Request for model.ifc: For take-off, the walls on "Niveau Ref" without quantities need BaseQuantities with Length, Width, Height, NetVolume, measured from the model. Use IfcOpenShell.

First a look at what the model holds.

```python
import ifcopenshell
import ifcopenshell.util.element
import ifcopenshell.util.unit

model = ifcopenshell.open("model.ifc")
print(model.schema)
for unit_type in ("LENGTHUNIT", "AREAUNIT", "VOLUMEUNIT"):
    print(unit_type, ifcopenshell.util.unit.calculate_unit_scale(model, unit_type))
storey = next(s for s in model.by_type("IfcBuildingStorey") if s.Name == "Niveau Ref")
walls = [e for e in ifcopenshell.util.element.get_decomposition(storey) if e.is_a("IfcWall")]
for e in sorted(walls, key=lambda e: e.id()):
    print(e.id(), e.is_a(), e.Name, list(ifcopenshell.util.element.get_psets(e, qtos_only=True)), sep=" | ")
```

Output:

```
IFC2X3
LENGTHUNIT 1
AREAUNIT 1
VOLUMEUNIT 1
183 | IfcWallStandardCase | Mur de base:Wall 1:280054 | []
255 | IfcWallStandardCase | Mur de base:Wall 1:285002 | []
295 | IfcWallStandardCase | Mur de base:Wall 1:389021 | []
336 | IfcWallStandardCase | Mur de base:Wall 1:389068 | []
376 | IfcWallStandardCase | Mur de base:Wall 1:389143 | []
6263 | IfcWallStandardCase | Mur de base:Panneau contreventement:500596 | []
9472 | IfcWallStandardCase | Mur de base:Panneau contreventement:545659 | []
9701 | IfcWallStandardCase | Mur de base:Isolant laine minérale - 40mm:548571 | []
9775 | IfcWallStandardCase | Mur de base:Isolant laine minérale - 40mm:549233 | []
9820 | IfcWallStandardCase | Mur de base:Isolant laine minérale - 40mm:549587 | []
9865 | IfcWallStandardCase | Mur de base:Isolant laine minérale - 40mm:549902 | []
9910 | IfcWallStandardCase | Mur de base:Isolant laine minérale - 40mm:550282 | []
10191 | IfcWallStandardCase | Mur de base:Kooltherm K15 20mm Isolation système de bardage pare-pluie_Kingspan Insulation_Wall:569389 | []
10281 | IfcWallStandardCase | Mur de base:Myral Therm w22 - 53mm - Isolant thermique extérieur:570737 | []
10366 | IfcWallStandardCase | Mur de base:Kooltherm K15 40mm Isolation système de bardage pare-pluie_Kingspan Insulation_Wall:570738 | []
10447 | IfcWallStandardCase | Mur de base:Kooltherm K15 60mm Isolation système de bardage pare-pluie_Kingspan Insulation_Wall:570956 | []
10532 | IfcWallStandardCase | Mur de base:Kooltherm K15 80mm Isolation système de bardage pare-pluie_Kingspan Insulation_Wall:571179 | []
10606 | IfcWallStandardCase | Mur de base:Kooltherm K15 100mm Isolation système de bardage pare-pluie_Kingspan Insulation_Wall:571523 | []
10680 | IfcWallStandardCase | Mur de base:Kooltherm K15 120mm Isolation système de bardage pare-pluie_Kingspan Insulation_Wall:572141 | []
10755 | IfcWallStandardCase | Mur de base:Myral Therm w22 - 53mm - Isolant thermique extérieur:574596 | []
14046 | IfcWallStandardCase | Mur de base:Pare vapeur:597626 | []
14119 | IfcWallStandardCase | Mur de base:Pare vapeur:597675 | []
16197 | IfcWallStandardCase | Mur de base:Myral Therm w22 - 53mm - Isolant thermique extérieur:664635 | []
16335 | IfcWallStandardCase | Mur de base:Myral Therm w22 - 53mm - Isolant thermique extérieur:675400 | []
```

```python
import ifcopenshell
import ifcopenshell.api.pset
import ifcopenshell.geom
import ifcopenshell.util.element
import ifcopenshell.util.shape
import ifcopenshell.util.unit

model = ifcopenshell.open("model.ifc")
unit_scale = ifcopenshell.util.unit.calculate_unit_scale(model)
volume_scale = ifcopenshell.util.unit.calculate_unit_scale(model, "VOLUMEUNIT")
settings = ifcopenshell.geom.settings()

storey = next(s for s in model.by_type("IfcBuildingStorey") if s.Name == "Niveau Ref")
walls = [e for e in ifcopenshell.util.element.get_decomposition(storey) if e.is_a("IfcWall")]

for e in sorted(walls, key=lambda e: e.id()):
    if ifcopenshell.util.element.get_psets(e, qtos_only=True, should_inherit=False):
        continue
    # Geometry comes back in metres, in the element's own axes.
    shape = ifcopenshell.geom.create_shape(settings, e)
    values = {
        "Length": ifcopenshell.util.shape.get_x(shape.geometry) / unit_scale,
        "Width": ifcopenshell.util.shape.get_y(shape.geometry) / unit_scale,
        "Height": ifcopenshell.util.shape.get_z(shape.geometry) / unit_scale,
        "NetVolume": ifcopenshell.util.shape.get_volume(shape.geometry) / volume_scale,
    }
    qto = ifcopenshell.api.pset.add_qto(model, product=e, name="BaseQuantities")
    ifcopenshell.api.pset.edit_qto(model, qto=qto, properties=values)
    print(e.id(), {k: round(v, 3) for k, v in values.items()})

model.write("model_updated.ifc")
```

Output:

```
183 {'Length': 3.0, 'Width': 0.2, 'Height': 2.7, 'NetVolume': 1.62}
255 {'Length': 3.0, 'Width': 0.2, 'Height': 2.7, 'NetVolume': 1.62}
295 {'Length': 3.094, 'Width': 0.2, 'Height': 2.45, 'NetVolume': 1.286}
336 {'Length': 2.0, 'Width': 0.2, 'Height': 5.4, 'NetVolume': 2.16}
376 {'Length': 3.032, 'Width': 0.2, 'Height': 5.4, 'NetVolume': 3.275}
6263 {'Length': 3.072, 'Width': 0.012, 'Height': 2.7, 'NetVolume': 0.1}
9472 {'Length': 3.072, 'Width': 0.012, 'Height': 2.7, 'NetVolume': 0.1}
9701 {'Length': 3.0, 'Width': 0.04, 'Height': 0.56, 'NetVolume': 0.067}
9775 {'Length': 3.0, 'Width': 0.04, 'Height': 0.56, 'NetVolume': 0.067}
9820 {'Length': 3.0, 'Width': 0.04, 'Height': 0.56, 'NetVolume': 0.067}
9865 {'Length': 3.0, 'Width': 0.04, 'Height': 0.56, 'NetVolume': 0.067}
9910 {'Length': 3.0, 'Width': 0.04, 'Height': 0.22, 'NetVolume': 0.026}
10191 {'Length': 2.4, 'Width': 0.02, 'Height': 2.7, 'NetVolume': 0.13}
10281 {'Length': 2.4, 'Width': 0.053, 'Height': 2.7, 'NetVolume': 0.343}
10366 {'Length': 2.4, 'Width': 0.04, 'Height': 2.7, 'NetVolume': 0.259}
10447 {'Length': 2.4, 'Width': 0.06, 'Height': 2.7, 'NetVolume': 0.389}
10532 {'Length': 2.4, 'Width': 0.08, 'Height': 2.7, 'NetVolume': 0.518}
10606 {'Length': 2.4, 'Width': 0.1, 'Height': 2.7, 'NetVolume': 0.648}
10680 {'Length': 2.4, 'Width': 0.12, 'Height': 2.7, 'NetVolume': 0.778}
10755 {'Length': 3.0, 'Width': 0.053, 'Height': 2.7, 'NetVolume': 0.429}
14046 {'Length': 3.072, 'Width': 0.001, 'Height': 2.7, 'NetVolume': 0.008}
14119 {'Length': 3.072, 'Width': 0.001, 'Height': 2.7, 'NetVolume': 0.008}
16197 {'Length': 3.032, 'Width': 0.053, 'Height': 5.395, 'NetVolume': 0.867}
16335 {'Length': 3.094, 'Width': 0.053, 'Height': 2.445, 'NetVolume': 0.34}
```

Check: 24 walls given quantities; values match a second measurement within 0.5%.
